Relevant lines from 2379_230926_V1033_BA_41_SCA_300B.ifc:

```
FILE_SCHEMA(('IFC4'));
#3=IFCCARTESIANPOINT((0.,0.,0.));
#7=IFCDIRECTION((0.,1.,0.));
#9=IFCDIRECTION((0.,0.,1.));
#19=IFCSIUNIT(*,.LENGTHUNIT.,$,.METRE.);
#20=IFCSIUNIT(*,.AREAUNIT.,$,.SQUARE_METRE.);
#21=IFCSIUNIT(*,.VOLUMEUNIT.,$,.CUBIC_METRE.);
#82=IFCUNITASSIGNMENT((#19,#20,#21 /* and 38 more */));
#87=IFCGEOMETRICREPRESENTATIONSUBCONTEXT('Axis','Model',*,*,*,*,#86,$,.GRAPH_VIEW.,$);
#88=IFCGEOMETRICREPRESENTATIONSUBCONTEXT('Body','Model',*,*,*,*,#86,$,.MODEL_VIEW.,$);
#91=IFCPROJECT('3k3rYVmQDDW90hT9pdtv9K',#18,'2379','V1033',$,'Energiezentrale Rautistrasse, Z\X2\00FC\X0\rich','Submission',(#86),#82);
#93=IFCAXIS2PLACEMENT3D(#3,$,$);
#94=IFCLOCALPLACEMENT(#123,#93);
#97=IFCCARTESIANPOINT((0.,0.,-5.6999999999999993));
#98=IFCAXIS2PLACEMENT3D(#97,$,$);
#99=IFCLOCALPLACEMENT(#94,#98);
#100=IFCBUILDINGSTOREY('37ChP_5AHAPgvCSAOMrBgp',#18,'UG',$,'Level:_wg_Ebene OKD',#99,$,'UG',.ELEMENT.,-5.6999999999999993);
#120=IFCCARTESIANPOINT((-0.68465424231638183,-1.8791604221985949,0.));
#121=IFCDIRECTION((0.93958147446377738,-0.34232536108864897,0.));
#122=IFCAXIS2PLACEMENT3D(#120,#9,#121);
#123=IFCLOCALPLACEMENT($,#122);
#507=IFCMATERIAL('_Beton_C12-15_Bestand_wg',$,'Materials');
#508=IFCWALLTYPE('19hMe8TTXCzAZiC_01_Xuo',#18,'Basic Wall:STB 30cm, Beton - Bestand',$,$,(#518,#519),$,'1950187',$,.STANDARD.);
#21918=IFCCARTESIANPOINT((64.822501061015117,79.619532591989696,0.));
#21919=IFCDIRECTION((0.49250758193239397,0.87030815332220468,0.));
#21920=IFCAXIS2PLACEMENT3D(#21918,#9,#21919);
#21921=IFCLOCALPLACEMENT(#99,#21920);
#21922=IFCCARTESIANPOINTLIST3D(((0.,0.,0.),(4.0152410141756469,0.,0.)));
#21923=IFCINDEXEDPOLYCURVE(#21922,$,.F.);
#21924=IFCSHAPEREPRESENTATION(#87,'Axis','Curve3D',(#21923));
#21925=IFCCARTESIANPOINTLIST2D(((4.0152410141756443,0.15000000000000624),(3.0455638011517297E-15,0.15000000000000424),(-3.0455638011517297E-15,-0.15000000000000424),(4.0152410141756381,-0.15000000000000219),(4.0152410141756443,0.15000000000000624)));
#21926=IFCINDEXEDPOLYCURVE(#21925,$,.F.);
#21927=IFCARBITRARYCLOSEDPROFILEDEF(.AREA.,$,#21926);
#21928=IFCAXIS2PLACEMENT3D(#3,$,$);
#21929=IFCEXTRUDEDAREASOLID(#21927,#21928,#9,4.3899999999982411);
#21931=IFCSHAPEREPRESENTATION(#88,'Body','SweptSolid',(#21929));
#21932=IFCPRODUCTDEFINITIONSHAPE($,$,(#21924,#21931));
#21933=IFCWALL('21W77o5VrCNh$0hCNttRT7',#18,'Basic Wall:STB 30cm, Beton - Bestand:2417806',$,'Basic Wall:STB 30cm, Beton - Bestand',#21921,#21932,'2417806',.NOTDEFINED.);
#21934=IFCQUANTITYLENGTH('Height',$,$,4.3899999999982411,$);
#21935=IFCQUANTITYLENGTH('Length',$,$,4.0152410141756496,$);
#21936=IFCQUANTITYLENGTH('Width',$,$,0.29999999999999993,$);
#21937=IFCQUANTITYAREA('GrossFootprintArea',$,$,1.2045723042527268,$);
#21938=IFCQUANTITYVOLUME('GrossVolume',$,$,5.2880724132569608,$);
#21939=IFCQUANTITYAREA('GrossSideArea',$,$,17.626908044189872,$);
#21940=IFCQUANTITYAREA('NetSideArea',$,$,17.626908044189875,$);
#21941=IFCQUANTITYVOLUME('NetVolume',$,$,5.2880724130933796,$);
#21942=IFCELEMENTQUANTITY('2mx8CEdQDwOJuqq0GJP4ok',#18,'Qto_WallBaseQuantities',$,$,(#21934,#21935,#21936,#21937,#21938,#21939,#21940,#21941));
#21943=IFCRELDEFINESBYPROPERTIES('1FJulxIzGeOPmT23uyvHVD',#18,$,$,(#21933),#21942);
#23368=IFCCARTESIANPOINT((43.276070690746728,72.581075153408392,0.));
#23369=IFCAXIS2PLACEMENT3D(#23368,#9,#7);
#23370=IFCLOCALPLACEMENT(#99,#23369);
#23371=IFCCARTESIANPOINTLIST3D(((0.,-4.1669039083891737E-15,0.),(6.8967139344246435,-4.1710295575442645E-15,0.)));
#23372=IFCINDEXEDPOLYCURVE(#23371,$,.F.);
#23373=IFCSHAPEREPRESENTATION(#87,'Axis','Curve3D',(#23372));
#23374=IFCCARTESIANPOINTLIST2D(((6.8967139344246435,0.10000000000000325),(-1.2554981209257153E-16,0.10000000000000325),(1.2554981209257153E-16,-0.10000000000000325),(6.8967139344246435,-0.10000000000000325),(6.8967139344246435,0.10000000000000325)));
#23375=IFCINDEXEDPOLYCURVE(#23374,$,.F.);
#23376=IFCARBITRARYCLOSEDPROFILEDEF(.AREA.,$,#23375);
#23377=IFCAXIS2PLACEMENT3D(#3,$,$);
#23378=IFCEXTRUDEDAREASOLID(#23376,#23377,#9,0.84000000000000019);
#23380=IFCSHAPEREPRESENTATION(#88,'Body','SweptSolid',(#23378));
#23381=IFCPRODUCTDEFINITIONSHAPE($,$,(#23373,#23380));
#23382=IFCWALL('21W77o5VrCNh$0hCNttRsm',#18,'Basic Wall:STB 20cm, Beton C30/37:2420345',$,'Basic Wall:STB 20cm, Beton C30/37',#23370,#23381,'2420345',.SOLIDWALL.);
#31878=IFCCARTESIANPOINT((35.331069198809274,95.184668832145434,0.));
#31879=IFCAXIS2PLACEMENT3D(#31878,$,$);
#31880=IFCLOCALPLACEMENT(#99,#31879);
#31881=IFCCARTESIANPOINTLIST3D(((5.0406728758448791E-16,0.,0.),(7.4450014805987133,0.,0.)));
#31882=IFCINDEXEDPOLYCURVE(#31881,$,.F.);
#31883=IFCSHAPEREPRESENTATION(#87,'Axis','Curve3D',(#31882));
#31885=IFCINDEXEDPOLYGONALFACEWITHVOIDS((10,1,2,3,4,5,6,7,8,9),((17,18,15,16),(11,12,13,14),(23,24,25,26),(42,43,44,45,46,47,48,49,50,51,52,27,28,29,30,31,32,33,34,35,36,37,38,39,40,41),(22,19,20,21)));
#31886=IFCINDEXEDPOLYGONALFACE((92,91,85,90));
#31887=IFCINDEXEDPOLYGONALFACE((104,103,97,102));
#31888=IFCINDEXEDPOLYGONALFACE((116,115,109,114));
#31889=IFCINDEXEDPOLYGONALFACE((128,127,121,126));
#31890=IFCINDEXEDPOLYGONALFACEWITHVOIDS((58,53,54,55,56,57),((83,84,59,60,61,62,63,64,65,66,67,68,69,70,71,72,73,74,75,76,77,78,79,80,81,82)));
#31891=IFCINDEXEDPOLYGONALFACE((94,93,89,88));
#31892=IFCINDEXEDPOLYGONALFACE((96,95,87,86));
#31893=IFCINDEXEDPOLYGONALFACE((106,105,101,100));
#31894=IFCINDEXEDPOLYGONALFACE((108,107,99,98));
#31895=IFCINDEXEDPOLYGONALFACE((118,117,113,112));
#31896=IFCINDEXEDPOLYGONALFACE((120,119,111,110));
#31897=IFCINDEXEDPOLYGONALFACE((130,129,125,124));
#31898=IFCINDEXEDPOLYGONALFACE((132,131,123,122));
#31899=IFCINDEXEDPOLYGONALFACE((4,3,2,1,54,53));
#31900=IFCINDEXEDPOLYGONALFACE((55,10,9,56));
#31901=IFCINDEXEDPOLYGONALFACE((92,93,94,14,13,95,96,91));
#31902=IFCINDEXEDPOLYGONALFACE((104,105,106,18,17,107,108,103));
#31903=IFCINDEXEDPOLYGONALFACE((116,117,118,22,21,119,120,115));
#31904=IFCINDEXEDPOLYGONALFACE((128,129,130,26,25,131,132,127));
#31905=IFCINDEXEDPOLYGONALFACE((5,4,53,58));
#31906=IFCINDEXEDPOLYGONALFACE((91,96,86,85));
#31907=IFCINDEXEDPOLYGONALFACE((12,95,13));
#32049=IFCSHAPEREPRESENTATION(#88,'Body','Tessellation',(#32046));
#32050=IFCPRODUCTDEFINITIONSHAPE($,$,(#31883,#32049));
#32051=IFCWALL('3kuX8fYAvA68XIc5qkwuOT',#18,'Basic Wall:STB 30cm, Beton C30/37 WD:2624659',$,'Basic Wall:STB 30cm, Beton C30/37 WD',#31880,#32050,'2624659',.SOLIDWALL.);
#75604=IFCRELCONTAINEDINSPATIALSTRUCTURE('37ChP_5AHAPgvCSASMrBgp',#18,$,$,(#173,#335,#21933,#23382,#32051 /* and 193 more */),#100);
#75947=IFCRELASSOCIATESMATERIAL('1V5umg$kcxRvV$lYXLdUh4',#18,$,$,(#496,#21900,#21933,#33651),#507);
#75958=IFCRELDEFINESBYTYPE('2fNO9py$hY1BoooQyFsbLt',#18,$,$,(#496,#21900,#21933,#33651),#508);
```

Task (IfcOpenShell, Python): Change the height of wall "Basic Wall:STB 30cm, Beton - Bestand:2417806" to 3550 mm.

```python
import ifcopenshell
import ifcopenshell.api.pset
import ifcopenshell.geom
import ifcopenshell.util.element
import ifcopenshell.util.representation
import ifcopenshell.util.shape
import ifcopenshell.util.unit

model = ifcopenshell.open("2379_230926_V1033_BA_41_SCA_300B.ifc")
unit_scale = ifcopenshell.util.unit.calculate_unit_scale(model)
area_scale = ifcopenshell.util.unit.calculate_unit_scale(model, "AREAUNIT")
volume_scale = ifcopenshell.util.unit.calculate_unit_scale(model, "VOLUMEUNIT")
settings = ifcopenshell.geom.settings()


def volume(element):
    """Net volume in cubic metres, openings subtracted."""
    shape = ifcopenshell.geom.create_shape(settings, element)
    return ifcopenshell.util.shape.get_volume(shape.geometry)


wall = model.by_guid("21W77o5VrCNh$0hCNttRT7")
before = volume(wall)

body = ifcopenshell.util.representation.get_representation(wall, "Model", "Body")
solid = body.Items[0]
old_height = solid.Depth
solid.Depth = 3.55 / unit_scale
after = volume(wall)
thickness = 0.3  # wall thickness in metres

# Update the stored height, areas and volumes.
qto = model.by_id(ifcopenshell.util.element.get_pset(wall, "Qto_WallBaseQuantities", should_inherit=False)["id"])
ifcopenshell.api.pset.edit_qto(model, qto=qto, properties={
    "Height": solid.Depth,
    "GrossVolume": ifcopenshell.util.element.get_pset(wall, "Qto_WallBaseQuantities", "GrossVolume") * solid.Depth / old_height,
    "GrossSideArea": ifcopenshell.util.element.get_pset(wall, "Qto_WallBaseQuantities", "GrossSideArea") * solid.Depth / old_height,
    "NetSideArea": after / thickness / area_scale,
    "NetVolume": after / volume_scale,
})

print(f"height {old_height:g} -> {solid.Depth:g}, volume {before:.3f} -> {after:.3f} m3")

model.write("2379_230926_V1033_BA_41_SCA_300B_updated.ifc")
```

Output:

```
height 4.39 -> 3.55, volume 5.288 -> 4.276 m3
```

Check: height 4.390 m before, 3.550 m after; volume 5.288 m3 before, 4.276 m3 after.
